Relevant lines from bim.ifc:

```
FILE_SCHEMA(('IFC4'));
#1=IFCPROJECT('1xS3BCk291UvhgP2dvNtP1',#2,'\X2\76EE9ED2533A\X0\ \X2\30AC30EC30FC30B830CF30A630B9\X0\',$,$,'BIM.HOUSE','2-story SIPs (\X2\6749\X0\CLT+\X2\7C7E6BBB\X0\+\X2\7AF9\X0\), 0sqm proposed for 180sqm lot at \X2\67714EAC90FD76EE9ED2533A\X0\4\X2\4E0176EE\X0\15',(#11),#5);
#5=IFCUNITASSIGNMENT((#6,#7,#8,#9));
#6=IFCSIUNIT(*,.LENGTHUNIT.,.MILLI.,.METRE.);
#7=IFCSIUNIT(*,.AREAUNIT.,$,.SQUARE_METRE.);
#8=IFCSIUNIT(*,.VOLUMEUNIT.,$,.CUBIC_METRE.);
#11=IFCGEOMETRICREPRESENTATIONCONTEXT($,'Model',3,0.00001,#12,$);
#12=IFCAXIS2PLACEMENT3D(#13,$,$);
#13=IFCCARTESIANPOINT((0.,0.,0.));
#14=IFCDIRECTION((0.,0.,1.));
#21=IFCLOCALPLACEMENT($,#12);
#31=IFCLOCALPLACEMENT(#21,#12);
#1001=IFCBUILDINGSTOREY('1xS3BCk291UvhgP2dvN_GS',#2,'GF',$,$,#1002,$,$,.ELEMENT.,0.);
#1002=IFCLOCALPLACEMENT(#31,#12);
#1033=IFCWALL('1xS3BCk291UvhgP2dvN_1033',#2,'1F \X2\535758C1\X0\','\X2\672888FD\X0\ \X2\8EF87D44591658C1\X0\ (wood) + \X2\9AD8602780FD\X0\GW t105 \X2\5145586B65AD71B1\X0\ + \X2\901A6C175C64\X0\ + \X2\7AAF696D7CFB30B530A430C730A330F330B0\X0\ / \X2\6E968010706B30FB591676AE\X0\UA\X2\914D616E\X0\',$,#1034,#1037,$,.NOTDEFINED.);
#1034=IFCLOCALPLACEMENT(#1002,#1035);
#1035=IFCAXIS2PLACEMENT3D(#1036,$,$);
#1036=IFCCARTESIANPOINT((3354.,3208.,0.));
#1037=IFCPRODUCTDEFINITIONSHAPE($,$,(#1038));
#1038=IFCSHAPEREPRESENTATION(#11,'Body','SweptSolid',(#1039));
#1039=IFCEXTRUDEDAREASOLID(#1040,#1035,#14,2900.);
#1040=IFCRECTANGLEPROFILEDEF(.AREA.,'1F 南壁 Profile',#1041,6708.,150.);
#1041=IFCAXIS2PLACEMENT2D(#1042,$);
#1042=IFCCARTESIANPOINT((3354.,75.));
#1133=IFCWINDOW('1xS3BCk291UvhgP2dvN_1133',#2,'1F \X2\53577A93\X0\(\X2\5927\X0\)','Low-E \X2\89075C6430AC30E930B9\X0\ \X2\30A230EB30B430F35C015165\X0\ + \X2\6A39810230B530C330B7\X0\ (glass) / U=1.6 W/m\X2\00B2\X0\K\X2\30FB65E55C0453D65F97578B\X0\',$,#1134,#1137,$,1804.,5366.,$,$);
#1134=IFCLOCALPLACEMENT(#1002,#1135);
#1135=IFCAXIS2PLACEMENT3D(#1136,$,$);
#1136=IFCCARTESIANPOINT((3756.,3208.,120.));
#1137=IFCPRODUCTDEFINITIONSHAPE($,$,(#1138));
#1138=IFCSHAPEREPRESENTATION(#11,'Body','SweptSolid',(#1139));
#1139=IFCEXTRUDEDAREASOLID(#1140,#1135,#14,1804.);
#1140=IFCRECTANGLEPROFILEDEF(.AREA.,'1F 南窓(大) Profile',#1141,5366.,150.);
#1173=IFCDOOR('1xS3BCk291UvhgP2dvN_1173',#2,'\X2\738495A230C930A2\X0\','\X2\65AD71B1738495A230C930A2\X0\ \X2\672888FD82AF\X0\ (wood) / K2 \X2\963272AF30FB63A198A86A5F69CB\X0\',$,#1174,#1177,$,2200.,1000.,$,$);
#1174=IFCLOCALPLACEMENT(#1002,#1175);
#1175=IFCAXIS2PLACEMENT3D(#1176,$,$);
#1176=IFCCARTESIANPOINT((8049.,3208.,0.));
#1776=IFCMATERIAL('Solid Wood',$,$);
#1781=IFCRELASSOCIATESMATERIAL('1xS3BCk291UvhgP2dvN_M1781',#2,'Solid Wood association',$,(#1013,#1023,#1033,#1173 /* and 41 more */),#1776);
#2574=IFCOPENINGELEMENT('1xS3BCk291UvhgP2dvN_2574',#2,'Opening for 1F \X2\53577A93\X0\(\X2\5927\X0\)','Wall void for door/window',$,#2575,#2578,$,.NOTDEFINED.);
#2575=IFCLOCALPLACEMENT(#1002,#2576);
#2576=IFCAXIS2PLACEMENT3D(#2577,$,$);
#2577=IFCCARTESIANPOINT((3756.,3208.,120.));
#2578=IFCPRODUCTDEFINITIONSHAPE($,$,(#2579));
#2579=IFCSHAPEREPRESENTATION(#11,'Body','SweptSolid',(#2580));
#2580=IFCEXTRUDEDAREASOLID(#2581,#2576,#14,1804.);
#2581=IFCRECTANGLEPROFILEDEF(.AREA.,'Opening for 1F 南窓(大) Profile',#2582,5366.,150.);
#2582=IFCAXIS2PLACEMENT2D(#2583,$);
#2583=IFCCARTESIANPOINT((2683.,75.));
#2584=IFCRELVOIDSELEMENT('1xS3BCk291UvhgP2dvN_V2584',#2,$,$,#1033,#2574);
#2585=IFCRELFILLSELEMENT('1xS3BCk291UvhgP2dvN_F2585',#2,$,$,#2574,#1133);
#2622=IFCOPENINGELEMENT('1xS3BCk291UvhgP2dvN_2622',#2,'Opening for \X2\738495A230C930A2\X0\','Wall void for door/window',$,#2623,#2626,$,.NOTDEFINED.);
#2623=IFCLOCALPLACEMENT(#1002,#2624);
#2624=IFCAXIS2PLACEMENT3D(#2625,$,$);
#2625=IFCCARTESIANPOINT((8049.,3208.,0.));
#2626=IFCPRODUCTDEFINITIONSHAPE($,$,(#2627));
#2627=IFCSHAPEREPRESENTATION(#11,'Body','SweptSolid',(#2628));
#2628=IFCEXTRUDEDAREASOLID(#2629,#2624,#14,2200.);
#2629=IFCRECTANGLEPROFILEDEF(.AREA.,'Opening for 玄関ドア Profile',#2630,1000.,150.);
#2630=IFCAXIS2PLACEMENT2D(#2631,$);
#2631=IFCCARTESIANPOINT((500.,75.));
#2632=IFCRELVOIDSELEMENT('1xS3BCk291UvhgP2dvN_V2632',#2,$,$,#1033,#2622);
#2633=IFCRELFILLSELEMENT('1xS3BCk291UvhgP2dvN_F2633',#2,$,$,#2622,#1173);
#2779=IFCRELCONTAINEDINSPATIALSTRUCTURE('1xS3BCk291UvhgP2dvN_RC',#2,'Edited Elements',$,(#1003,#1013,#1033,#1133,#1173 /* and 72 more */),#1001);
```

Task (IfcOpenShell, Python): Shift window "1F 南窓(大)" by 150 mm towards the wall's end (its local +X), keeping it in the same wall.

```python
import ifcopenshell
import ifcopenshell.api.geometry
import ifcopenshell.util.placement

model = ifcopenshell.open("bim.ifc")

window = model.by_guid("1xS3BCk291UvhgP2dvN_1133")
opening = window.FillsVoids[0].RelatingOpeningElement
wall = opening.VoidsElements[0].RelatingBuildingElement

wall_matrix = ifcopenshell.util.placement.get_local_placement(wall.ObjectPlacement)
shift = wall_matrix[:3, 0] * 150.0
before = ifcopenshell.util.placement.get_local_placement(window.ObjectPlacement)[:3, 3].copy()

# The window is not placed relative to its opening, so move both.
for product in (opening, window):
    matrix = ifcopenshell.util.placement.get_local_placement(product.ObjectPlacement)
    matrix[:3, 3] += shift
    ifcopenshell.api.geometry.edit_object_placement(model, product=product, matrix=matrix, is_si=False)

after = ifcopenshell.util.placement.get_local_placement(window.ObjectPlacement)[:3, 3]
print("window moved by", (after - before).round(3) + 0.0)

model.write("bim-out.ifc")
```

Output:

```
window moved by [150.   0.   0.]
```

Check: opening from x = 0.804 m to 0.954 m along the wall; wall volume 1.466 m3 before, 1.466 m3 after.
